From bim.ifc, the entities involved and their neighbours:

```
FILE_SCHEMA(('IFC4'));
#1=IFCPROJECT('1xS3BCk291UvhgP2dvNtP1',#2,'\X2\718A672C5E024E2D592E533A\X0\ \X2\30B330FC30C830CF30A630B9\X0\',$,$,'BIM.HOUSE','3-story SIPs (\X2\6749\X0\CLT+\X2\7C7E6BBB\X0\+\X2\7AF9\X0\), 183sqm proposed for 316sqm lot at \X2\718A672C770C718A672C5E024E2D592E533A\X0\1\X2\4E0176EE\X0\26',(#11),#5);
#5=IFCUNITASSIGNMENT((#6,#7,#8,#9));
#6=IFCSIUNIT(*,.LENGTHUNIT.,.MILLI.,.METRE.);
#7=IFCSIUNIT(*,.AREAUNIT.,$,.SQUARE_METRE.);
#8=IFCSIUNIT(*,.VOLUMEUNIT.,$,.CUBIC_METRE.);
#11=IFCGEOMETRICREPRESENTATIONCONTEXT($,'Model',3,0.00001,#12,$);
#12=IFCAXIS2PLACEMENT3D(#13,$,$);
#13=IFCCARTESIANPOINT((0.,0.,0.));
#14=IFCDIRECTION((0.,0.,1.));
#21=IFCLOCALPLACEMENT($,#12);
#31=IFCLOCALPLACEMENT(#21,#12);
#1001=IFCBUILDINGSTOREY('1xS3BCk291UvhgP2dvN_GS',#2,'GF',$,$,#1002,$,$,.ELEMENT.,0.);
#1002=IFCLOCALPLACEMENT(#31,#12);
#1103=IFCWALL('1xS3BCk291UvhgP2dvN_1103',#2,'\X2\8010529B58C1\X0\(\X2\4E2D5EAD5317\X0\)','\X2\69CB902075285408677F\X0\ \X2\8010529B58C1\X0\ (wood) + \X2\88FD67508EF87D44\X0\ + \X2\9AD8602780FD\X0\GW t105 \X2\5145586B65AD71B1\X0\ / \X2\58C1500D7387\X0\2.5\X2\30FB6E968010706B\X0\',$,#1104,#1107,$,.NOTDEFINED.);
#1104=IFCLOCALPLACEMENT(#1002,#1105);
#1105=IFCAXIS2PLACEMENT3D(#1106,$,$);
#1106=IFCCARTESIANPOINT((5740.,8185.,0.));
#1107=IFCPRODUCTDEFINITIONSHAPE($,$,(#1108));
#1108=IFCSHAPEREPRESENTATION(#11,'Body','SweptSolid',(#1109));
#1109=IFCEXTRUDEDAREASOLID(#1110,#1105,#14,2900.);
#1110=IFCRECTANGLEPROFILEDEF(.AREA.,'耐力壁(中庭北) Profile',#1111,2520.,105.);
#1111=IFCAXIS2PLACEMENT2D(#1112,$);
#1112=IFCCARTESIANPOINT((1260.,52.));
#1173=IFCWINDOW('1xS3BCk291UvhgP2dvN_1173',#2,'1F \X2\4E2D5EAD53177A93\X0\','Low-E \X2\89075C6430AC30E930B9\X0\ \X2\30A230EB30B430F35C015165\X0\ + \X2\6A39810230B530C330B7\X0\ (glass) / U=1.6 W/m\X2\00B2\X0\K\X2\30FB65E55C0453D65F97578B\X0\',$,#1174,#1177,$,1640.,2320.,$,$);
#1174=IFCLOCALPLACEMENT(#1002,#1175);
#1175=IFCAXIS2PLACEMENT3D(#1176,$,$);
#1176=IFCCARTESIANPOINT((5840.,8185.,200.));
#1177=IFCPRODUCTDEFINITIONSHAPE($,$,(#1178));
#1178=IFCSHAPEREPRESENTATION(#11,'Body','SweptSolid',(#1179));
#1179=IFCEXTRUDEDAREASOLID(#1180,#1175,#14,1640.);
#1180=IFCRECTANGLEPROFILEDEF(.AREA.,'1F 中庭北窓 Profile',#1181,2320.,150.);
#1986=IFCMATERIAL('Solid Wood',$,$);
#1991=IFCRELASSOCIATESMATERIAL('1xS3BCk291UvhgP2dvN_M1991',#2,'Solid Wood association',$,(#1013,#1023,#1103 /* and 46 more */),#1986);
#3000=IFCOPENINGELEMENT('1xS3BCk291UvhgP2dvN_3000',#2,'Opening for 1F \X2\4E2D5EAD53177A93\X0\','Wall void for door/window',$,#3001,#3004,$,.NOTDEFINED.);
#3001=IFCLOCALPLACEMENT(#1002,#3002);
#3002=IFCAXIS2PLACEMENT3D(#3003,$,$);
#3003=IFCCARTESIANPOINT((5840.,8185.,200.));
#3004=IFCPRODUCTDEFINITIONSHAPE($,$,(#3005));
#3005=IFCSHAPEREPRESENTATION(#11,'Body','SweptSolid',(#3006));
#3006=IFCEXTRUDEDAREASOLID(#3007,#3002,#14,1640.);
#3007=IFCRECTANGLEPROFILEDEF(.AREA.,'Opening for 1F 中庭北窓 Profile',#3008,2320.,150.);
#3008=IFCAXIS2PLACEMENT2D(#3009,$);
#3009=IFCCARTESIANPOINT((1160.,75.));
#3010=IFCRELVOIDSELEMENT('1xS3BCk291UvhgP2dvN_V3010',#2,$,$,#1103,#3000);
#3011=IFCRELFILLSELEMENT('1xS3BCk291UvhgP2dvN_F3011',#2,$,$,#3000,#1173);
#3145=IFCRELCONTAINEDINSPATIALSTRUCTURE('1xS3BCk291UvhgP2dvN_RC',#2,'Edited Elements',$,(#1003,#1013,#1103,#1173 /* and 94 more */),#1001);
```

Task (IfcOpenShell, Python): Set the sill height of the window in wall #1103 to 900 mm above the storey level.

```python
import numpy as np
import ifcopenshell
import ifcopenshell.api.geometry
import ifcopenshell.geom
import ifcopenshell.util.element
import ifcopenshell.util.placement
import ifcopenshell.util.shape
import ifcopenshell.util.unit

model = ifcopenshell.open("bim.ifc")
unit_scale = ifcopenshell.util.unit.calculate_unit_scale(model)

window = model.by_guid("1xS3BCk291UvhgP2dvN_1173")
opening = window.FillsVoids[0].RelatingOpeningElement
storey = ifcopenshell.util.element.get_container(window, ifc_class="IfcBuildingStorey")
level = ifcopenshell.util.placement.get_local_placement(storey.ObjectPlacement)[2, 3]

# The opening's origin need not be at the sill, so measure its lowest point.
shape = ifcopenshell.geom.create_shape(ifcopenshell.geom.settings(), opening)
bottom = ifcopenshell.util.shape.get_shape_bottom_elevation(shape, shape.geometry) / unit_scale
dz = level + 0.9 / unit_scale - bottom

shift = np.array([0.0, 0.0, dz])
# The window is not placed relative to its opening, so move both.
for product in (opening, window):
    matrix = ifcopenshell.util.placement.get_local_placement(product.ObjectPlacement)
    matrix[:3, 3] += shift
    ifcopenshell.api.geometry.edit_object_placement(model, product=product, matrix=matrix, is_si=False)

print(f"moved by {dz * unit_scale:+.3f} m")

model.write("bim-out.ifc")
```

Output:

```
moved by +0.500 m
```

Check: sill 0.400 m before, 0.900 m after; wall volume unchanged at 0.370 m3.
